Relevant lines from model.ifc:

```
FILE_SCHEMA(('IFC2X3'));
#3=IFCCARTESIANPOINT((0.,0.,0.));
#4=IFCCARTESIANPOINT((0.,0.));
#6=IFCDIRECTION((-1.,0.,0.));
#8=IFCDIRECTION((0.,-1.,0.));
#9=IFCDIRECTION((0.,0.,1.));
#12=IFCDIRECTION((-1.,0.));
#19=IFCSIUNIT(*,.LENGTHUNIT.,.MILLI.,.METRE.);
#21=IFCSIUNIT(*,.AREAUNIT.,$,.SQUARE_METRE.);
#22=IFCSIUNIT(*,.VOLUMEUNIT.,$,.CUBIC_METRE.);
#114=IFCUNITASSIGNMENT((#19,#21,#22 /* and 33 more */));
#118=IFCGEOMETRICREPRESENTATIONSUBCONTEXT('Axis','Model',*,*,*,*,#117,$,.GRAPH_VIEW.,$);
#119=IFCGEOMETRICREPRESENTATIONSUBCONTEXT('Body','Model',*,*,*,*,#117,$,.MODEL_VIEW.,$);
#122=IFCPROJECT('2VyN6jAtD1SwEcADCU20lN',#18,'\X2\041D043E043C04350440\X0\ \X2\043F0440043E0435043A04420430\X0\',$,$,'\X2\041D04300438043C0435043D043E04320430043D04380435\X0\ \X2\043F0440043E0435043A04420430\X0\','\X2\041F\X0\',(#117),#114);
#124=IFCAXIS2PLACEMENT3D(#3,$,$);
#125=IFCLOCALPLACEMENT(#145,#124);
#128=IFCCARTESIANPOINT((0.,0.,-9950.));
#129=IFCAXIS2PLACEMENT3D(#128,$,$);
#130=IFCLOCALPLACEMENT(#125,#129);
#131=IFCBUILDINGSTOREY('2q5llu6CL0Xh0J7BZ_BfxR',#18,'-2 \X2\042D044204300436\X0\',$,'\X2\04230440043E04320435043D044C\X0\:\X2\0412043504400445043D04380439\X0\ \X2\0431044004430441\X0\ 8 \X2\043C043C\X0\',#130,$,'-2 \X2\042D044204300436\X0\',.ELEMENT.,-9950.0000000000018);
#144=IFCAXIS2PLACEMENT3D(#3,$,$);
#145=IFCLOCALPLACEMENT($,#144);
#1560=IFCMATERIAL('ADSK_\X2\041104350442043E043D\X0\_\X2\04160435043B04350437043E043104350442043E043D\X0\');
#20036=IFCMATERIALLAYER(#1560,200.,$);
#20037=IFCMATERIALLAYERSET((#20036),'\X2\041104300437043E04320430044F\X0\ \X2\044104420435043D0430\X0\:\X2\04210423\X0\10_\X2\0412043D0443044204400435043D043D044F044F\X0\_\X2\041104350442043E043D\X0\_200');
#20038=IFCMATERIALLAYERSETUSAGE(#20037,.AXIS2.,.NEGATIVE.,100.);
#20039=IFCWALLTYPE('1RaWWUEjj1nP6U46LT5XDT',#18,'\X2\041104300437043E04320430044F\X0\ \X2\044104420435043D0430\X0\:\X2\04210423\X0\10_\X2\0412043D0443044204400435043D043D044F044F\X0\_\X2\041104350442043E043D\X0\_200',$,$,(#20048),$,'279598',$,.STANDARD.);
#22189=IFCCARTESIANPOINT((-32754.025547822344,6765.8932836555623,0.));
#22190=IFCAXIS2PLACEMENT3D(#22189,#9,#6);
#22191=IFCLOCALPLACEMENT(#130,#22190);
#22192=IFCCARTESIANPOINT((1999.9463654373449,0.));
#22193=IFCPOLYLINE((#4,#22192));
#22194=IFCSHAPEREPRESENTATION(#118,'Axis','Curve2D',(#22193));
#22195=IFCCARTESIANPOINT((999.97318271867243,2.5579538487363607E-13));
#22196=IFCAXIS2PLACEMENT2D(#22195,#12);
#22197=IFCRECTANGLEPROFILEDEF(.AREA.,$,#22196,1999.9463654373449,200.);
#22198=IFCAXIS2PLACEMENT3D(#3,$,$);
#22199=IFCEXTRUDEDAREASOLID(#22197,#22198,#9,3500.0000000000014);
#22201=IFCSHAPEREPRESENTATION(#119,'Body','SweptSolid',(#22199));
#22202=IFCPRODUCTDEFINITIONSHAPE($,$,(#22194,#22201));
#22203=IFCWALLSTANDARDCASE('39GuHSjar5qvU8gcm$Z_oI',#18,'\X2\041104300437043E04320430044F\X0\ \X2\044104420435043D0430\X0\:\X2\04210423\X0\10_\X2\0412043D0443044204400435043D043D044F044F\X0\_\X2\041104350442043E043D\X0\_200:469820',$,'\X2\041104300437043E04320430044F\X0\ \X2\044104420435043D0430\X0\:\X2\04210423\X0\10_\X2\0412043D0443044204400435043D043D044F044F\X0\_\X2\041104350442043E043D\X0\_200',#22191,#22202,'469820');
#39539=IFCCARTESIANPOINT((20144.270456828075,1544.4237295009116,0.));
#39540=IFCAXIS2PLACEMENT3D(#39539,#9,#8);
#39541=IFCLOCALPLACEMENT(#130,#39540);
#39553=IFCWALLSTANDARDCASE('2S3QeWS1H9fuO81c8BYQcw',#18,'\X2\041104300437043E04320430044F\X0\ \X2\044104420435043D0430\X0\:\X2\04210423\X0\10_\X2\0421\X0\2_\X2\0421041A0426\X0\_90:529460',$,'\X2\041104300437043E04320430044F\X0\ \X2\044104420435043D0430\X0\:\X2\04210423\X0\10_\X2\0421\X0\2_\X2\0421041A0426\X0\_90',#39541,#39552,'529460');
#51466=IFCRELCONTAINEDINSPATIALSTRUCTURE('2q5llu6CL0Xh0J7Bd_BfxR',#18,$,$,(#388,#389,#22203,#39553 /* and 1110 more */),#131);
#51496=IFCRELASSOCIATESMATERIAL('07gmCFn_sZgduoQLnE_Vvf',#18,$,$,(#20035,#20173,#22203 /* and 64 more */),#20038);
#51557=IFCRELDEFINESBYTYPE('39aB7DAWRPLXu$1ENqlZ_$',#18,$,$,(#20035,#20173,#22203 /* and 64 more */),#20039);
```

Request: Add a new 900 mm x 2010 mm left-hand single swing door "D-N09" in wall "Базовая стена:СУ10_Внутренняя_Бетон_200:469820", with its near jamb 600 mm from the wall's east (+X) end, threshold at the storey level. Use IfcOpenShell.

```python
import numpy as np
import ifcopenshell
import ifcopenshell.api.feature
import ifcopenshell.api.geometry
import ifcopenshell.api.root
import ifcopenshell.api.spatial
import ifcopenshell.api.type
import ifcopenshell.geom
import ifcopenshell.util.element
import ifcopenshell.util.placement
import ifcopenshell.util.representation
import ifcopenshell.util.shape
import ifcopenshell.util.unit

model = ifcopenshell.open("model.ifc")
unit_scale = ifcopenshell.util.unit.calculate_unit_scale(model)
settings = ifcopenshell.geom.settings()


def volume(element):
    """Net volume in cubic metres, openings subtracted."""
    shape = ifcopenshell.geom.create_shape(settings, element)
    return ifcopenshell.util.shape.get_volume(shape.geometry)


wall = model.by_guid("39GuHSjar5qvU8gcm$Z_oI")
storey = ifcopenshell.util.element.get_container(wall, ifc_class="IfcBuildingStorey")
context = ifcopenshell.util.representation.get_context(model, "Model", "Body", "MODEL_VIEW")
before = volume(wall)

width, height, from_end, sill = 0.9, 2.01, 0.6, 0.0  # metres

# The wall runs along its own X axis, and the end named is its -X end.
wall_shape = ifcopenshell.geom.create_shape(settings, wall)
x, y, z = ifcopenshell.util.shape.get_vertices(wall_shape.geometry).T
start = x.min() + from_end
face, thickness = float(y.min()), float(y.max() - y.min())
wall_matrix = ifcopenshell.util.placement.get_local_placement(wall.ObjectPlacement)
level = ifcopenshell.util.placement.get_local_placement(storey.ObjectPlacement)[2, 3]


def in_wall(x, y):
    """Placement at x, y metres in the wall's axes, at sill height."""
    matrix = wall_matrix.copy()
    matrix[:, 3] = wall_matrix @ np.array([x / unit_scale, y / unit_scale, 0.0, 1.0])
    matrix[2, 3] = level + sill / unit_scale
    return matrix


# Opening: a box that overshoots both wall faces by 50 mm.
opening = ifcopenshell.api.root.create_entity(model, ifc_class="IfcOpeningElement")
box = ifcopenshell.api.geometry.add_wall_representation(
    model, context=context, length=width, height=height, thickness=thickness + 0.1
)
ifcopenshell.api.geometry.assign_representation(model, product=opening, representation=box)
ifcopenshell.api.geometry.edit_object_placement(model, product=opening, matrix=in_wall(start, face - 0.05), is_si=False)
ifcopenshell.api.feature.add_feature(model, feature=opening, element=wall)

door = ifcopenshell.api.root.create_entity(model, ifc_class="IfcDoor", name="D-N09")
door.OverallWidth, door.OverallHeight = width / unit_scale, height / unit_scale
body = ifcopenshell.api.geometry.add_door_representation(
    model,
    context=context,
    overall_width=door.OverallWidth,
    overall_height=door.OverallHeight,
    operation_type="SINGLE_SWING_LEFT",
    lining_properties={"LiningDepth": thickness / unit_scale, "ThresholdDepth": thickness / unit_scale},
)
ifcopenshell.api.geometry.assign_representation(model, product=door, representation=body)
ifcopenshell.api.spatial.assign_container(model, products=[door], relating_structure=storey)
fills = ifcopenshell.api.feature.add_filling(model, opening=opening, element=door)
fills.OwnerHistory = door.OwnerHistory  # required in IFC2X3

# IFC2X3 keeps the operation on the door style.
style = ifcopenshell.api.root.create_entity(model, ifc_class="IfcDoorStyle", name="D-N09")
style.OperationType, style.ConstructionType = "SINGLE_SWING_LEFT", "NOTDEFINED"
style.ParameterTakesPrecedence = style.Sizeable = False
ifcopenshell.api.type.assign_type(model, related_objects=[door], relating_type=style)

# The lining spans the wall, so the door starts at the wall face.
ifcopenshell.api.geometry.edit_object_placement(model, product=door, matrix=in_wall(start, face), is_si=False)

after = volume(wall)

print(f"wall volume {before:.3f} -> {after:.3f} m3")

model.write("model_updated.ifc")
```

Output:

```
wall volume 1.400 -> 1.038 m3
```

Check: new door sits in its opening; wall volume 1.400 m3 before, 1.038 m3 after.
